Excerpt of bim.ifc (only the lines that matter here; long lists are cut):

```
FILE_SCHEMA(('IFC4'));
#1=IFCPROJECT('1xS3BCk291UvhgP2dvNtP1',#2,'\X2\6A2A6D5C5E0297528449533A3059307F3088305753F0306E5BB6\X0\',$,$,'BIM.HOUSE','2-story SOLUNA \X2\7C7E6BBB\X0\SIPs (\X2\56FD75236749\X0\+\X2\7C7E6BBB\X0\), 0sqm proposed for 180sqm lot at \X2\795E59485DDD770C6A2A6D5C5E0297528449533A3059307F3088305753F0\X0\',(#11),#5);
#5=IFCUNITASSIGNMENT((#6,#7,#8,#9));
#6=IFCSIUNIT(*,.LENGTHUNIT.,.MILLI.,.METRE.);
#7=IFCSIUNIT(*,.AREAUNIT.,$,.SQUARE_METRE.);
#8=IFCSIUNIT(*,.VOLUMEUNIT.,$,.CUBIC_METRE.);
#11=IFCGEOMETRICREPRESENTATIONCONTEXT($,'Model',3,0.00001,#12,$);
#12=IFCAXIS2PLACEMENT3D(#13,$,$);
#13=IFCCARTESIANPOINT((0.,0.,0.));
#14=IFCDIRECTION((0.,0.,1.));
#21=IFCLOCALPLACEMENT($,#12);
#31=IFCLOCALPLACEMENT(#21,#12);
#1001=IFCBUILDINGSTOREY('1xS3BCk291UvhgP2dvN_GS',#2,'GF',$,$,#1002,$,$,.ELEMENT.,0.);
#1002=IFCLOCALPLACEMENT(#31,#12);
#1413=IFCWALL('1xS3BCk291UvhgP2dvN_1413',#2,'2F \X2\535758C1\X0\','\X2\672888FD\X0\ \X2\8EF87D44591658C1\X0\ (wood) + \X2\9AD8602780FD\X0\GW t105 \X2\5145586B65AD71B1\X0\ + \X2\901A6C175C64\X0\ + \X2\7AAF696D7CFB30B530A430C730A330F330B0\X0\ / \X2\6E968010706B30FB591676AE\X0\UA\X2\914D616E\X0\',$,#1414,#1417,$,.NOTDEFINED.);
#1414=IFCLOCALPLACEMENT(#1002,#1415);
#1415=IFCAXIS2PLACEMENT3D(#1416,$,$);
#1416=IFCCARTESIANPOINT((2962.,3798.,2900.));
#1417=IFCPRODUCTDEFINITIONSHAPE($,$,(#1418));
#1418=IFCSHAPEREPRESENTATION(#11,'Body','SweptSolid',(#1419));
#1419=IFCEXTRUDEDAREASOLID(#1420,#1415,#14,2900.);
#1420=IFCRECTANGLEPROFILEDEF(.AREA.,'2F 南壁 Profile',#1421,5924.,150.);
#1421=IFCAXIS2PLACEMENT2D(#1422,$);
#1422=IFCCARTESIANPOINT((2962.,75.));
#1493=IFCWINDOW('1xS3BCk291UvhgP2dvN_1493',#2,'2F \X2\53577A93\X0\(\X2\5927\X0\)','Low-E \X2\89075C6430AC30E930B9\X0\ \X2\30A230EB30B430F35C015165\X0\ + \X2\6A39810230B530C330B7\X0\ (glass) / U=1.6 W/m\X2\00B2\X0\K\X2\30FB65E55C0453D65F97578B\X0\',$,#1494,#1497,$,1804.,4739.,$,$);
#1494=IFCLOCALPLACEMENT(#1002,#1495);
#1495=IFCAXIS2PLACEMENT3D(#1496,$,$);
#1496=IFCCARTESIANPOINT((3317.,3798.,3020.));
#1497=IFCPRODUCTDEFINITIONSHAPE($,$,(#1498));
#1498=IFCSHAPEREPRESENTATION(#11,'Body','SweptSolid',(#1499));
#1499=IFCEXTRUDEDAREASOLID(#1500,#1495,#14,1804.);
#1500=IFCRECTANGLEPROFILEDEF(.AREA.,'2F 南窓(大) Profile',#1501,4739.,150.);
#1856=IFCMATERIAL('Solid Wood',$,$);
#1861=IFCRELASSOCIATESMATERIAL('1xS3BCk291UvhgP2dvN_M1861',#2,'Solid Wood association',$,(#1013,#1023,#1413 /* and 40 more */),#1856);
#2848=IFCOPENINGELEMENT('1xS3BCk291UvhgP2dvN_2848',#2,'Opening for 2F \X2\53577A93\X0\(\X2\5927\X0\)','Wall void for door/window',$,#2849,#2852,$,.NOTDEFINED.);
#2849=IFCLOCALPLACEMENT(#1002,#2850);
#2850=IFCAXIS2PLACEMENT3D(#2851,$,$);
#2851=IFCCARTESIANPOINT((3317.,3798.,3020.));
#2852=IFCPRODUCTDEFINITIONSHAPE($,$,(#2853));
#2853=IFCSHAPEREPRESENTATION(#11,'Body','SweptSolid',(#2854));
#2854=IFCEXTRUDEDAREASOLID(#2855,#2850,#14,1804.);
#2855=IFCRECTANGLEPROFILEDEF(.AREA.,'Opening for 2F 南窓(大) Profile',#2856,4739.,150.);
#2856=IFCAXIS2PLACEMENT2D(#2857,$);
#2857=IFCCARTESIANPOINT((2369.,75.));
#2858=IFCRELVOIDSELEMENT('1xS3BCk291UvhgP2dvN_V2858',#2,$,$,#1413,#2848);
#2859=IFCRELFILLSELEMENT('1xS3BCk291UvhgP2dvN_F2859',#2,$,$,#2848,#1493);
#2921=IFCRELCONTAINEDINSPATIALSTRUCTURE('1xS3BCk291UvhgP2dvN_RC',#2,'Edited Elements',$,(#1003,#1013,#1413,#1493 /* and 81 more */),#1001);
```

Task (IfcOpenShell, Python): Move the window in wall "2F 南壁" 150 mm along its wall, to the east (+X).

```python
import ifcopenshell
import ifcopenshell.api.geometry
import ifcopenshell.util.placement
import ifcopenshell.util.unit

model = ifcopenshell.open("bim.ifc")
unit_scale = ifcopenshell.util.unit.calculate_unit_scale(model)

window = model.by_guid("1xS3BCk291UvhgP2dvN_1493")
opening = window.FillsVoids[0].RelatingOpeningElement
wall = opening.VoidsElements[0].RelatingBuildingElement

wall_matrix = ifcopenshell.util.placement.get_local_placement(wall.ObjectPlacement)
shift = wall_matrix[:3, 0] * 0.15 / unit_scale
before = ifcopenshell.util.placement.get_local_placement(window.ObjectPlacement)[:3, 3].copy()

# The window is not placed relative to its opening, so move both.
for product in (opening, window):
    matrix = ifcopenshell.util.placement.get_local_placement(product.ObjectPlacement)
    matrix[:3, 3] += shift
    ifcopenshell.api.geometry.edit_object_placement(model, product=product, matrix=matrix, is_si=False)

after = ifcopenshell.util.placement.get_local_placement(window.ObjectPlacement)[:3, 3]
print("window moved by", (after - before).round(3) + 0.0)

model.write("bim-out.ifc")
```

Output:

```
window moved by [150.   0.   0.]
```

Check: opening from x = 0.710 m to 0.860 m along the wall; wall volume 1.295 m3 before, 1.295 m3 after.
